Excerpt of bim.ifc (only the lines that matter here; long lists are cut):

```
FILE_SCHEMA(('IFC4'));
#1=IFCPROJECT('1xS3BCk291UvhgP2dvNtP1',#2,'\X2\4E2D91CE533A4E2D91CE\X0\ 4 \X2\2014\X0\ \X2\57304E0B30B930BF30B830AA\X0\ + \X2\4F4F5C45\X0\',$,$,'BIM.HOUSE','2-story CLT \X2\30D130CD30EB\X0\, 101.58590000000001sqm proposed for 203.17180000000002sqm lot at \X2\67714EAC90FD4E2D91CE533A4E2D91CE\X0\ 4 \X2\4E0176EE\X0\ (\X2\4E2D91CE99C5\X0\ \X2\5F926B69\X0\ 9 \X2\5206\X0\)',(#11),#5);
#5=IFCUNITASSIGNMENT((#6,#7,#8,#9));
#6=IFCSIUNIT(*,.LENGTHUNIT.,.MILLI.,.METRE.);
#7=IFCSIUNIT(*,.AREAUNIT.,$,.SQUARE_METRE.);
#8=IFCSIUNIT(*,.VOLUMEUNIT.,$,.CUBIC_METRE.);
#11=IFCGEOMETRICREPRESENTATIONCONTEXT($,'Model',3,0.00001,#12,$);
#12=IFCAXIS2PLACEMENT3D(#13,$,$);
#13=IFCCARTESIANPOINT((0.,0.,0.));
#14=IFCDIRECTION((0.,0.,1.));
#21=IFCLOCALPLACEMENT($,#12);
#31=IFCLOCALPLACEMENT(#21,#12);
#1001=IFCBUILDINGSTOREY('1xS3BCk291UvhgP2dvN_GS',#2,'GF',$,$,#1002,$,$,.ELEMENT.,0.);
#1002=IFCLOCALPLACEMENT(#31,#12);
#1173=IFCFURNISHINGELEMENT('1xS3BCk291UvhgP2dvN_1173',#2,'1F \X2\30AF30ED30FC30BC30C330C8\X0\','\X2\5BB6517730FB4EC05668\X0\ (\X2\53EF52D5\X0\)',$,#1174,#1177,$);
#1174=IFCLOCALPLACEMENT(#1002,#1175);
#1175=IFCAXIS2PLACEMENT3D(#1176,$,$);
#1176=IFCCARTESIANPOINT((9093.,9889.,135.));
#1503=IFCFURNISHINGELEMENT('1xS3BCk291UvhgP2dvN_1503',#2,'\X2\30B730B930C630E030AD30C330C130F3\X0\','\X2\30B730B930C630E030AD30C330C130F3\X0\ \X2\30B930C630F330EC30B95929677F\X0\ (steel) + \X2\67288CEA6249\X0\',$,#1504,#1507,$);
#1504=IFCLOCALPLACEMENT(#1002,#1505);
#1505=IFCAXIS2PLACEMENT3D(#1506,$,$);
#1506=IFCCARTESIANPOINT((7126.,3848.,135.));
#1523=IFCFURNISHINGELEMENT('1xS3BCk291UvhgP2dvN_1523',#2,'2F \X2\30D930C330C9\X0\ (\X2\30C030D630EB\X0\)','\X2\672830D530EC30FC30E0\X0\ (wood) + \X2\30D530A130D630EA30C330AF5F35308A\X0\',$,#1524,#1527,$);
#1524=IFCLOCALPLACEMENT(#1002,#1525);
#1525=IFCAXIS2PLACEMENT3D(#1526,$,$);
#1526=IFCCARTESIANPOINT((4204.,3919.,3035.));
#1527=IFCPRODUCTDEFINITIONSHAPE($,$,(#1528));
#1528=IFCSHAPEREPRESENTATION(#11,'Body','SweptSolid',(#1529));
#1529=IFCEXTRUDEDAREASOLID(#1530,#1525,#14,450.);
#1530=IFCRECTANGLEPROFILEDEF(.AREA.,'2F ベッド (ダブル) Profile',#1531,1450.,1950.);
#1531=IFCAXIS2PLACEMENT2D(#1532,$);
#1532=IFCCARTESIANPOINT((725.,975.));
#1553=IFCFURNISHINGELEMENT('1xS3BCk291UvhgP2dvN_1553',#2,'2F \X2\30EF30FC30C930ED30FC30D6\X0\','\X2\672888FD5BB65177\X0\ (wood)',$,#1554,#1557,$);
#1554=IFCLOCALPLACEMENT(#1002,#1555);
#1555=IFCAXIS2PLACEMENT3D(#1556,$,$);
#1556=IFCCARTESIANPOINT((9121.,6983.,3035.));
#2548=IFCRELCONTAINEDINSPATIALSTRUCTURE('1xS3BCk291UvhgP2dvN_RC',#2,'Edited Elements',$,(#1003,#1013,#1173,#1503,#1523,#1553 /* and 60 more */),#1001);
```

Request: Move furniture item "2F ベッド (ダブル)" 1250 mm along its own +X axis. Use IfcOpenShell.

```python
import ifcopenshell
import ifcopenshell.api.geometry
import ifcopenshell.util.placement

model = ifcopenshell.open("bim.ifc")

item = model.by_guid("1xS3BCk291UvhgP2dvN_1523")
matrix = ifcopenshell.util.placement.get_local_placement(item.ObjectPlacement)
matrix[:3, 3] += matrix[:3, 0] * 1250.0
ifcopenshell.api.geometry.edit_object_placement(model, product=item, matrix=matrix, is_si=False)

print(ifcopenshell.util.placement.get_local_placement(item.ObjectPlacement).round(3) + 0.0)

model.write("bim_updated.ifc")
```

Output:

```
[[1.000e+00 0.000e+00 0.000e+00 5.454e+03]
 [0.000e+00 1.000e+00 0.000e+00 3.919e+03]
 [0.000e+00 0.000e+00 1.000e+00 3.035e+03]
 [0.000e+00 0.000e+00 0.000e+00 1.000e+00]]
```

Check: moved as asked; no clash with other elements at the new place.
